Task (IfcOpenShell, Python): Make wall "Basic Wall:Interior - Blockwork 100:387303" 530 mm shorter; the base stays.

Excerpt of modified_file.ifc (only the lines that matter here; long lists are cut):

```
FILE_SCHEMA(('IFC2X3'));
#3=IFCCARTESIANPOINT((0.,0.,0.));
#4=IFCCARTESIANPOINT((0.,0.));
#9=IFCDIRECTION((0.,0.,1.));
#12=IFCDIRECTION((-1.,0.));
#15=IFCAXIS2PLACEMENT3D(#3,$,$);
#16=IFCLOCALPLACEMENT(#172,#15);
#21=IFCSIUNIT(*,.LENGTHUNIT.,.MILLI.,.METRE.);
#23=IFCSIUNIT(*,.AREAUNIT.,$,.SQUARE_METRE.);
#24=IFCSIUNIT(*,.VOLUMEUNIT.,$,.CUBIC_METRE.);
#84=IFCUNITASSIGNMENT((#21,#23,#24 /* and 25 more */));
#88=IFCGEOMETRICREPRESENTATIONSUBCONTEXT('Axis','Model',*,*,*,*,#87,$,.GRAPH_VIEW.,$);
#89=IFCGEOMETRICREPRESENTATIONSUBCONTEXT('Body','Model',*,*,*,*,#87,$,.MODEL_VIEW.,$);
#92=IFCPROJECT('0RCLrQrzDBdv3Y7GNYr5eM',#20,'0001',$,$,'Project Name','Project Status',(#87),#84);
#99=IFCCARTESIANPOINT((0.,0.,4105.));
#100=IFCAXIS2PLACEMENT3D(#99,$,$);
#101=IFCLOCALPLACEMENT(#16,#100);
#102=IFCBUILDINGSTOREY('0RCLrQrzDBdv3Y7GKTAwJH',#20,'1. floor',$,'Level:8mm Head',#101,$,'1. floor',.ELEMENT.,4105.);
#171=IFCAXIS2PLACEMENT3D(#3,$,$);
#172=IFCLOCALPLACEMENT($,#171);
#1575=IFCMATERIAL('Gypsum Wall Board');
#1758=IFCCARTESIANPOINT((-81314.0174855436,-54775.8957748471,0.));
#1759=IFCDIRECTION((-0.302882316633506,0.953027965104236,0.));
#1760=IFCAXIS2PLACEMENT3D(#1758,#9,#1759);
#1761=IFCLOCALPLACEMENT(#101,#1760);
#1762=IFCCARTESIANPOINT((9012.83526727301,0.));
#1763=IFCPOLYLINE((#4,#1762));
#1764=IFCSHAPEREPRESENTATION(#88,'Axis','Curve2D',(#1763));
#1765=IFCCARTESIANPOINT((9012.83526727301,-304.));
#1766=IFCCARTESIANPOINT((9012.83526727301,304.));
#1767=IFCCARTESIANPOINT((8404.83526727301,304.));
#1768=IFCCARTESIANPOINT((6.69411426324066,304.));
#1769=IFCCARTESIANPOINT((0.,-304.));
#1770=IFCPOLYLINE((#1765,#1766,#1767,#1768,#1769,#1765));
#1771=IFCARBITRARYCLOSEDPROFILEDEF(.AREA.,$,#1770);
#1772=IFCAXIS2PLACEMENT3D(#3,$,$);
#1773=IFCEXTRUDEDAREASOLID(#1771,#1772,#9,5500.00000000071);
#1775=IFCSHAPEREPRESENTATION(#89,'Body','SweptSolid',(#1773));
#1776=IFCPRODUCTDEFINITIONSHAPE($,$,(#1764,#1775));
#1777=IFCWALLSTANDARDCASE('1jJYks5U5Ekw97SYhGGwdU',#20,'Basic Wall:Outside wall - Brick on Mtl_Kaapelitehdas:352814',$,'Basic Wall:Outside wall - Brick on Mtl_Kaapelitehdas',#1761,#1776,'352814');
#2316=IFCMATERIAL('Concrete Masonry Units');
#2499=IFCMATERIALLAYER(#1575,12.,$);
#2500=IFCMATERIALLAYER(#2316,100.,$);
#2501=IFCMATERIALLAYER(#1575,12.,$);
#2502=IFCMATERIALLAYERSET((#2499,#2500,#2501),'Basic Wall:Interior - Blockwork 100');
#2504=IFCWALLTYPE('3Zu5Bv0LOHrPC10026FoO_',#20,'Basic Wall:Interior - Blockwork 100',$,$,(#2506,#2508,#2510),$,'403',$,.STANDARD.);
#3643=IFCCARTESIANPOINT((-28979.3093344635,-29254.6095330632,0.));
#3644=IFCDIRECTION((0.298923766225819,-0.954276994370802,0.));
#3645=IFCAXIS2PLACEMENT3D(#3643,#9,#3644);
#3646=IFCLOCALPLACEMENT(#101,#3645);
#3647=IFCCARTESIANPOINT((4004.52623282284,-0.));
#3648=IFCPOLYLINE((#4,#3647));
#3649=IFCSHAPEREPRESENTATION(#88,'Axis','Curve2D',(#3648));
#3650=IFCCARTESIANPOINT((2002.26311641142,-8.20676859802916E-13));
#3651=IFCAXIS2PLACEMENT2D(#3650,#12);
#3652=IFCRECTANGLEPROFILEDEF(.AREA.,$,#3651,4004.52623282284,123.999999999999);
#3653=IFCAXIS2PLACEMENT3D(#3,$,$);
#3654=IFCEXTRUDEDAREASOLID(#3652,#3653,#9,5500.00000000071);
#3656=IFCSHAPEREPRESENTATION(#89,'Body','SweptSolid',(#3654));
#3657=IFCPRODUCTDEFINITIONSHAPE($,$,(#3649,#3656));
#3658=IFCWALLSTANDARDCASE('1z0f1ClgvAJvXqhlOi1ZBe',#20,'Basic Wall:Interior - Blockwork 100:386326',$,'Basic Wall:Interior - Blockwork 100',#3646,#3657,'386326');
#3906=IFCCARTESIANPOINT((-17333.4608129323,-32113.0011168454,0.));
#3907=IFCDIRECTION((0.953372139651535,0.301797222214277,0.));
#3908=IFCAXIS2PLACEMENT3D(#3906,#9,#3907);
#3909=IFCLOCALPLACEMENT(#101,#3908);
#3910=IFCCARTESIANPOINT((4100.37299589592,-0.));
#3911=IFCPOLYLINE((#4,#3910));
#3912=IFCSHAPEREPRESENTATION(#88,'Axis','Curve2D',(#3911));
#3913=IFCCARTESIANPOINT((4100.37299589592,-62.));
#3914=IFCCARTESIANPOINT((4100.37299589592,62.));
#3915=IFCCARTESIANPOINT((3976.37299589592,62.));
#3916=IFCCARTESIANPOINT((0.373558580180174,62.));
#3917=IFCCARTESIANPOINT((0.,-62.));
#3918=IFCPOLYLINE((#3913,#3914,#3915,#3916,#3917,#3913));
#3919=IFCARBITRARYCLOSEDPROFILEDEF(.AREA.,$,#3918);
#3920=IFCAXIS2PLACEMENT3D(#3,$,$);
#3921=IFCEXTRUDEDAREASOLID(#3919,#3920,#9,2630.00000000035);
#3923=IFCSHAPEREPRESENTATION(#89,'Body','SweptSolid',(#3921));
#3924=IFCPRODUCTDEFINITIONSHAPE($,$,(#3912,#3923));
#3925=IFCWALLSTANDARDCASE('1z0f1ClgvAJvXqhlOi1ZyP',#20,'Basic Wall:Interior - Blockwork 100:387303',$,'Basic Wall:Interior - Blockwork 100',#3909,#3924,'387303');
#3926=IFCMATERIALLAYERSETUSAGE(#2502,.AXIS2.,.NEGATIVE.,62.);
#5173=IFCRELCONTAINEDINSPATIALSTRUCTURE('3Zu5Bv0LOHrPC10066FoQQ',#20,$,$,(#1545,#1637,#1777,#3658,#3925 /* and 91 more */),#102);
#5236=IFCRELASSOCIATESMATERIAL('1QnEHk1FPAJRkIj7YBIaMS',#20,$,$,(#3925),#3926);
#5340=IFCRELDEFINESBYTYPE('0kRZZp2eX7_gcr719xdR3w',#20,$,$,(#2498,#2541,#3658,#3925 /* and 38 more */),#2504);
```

```python
import ifcopenshell
import ifcopenshell.geom
import ifcopenshell.util.representation
import ifcopenshell.util.shape

model = ifcopenshell.open("modified_file.ifc")
settings = ifcopenshell.geom.settings()


def volume(element):
    """Net volume in cubic metres, openings subtracted."""
    shape = ifcopenshell.geom.create_shape(settings, element)
    return ifcopenshell.util.shape.get_volume(shape.geometry)


wall = model.by_guid("1z0f1ClgvAJvXqhlOi1ZyP")
before = volume(wall)

body = ifcopenshell.util.representation.get_representation(wall, "Model", "Body")
solid = body.Items[0]
old_height = solid.Depth
solid.Depth -= 530.0
after = volume(wall)

print(f"height {old_height:g} -> {solid.Depth:g}, volume {before:.3f} -> {after:.3f} m3")

model.write("modified_file-out.ifc")
```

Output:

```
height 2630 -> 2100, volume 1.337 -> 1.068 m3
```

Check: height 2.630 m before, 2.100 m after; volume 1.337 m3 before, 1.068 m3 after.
